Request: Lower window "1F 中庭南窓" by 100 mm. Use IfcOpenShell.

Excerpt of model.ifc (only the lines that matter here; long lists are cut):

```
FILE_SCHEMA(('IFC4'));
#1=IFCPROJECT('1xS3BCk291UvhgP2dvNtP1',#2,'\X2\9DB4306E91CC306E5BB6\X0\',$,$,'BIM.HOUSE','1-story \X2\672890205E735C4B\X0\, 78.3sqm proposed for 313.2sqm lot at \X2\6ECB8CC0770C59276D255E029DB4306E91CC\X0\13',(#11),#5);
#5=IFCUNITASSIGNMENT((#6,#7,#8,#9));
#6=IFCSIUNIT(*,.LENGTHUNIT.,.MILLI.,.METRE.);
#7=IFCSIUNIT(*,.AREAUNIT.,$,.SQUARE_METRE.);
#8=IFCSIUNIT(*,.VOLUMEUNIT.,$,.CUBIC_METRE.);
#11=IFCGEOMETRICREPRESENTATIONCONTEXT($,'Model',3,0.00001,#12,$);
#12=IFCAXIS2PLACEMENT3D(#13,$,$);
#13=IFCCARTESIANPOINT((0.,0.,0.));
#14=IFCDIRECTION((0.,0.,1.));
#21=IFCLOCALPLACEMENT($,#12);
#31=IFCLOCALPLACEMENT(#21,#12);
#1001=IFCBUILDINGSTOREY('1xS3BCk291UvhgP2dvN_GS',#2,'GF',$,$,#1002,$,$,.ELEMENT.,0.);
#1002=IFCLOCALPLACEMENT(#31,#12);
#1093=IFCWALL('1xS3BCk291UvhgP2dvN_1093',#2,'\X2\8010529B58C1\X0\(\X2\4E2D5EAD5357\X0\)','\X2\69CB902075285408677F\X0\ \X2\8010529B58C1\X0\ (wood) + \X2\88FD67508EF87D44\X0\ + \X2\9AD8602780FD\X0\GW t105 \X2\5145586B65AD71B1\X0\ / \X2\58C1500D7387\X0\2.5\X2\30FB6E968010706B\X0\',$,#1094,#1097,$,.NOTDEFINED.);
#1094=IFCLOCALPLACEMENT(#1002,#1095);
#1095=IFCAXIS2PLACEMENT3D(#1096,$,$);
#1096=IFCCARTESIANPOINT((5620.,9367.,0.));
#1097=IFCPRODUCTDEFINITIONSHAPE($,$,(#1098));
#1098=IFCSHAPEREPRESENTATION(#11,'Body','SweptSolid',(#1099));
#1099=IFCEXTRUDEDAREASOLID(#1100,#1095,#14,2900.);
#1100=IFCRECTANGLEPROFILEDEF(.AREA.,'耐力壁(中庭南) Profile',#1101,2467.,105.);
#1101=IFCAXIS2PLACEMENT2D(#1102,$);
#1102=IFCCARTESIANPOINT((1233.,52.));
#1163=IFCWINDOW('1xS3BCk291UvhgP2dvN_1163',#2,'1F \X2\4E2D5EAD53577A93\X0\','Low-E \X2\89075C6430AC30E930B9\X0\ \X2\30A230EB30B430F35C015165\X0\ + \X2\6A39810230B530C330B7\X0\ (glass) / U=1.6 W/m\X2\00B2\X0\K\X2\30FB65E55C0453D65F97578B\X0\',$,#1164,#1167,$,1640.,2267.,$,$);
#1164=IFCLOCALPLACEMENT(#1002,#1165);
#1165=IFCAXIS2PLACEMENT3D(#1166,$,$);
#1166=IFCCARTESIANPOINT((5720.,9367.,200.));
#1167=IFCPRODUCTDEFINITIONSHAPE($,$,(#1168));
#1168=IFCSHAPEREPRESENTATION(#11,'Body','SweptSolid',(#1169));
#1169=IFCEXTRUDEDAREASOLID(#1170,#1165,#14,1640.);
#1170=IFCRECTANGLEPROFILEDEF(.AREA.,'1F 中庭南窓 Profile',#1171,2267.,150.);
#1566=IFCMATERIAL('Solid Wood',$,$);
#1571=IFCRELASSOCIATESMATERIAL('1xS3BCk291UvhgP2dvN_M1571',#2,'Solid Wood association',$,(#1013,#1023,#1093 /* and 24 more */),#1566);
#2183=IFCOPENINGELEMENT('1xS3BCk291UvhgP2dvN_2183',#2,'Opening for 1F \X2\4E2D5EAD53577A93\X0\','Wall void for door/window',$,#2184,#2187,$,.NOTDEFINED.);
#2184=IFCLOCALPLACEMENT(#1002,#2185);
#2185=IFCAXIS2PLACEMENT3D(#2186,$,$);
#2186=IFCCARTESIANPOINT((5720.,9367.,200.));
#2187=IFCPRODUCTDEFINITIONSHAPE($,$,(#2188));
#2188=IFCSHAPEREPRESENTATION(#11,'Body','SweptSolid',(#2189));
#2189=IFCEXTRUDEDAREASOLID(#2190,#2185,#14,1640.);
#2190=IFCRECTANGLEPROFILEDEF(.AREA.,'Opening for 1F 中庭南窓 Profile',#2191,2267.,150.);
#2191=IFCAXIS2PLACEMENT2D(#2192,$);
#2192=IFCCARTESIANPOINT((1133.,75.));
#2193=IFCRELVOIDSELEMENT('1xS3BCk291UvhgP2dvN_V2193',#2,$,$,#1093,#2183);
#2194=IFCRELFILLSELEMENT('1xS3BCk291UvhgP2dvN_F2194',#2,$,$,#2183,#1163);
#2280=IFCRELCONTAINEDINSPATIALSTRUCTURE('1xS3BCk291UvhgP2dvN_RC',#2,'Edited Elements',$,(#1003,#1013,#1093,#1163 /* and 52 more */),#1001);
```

```python
import numpy as np
import ifcopenshell
import ifcopenshell.api.geometry
import ifcopenshell.util.placement
import ifcopenshell.util.unit

model = ifcopenshell.open("model.ifc")
unit_scale = ifcopenshell.util.unit.calculate_unit_scale(model)

window = model.by_id(1163)
opening = window.FillsVoids[0].RelatingOpeningElement
dz = -0.1 / unit_scale

shift = np.array([0.0, 0.0, dz])
# The window is not placed relative to its opening, so move both.
for product in (opening, window):
    matrix = ifcopenshell.util.placement.get_local_placement(product.ObjectPlacement)
    matrix[:3, 3] += shift
    ifcopenshell.api.geometry.edit_object_placement(model, product=product, matrix=matrix, is_si=False)

print(f"moved by {dz * unit_scale:+.3f} m")

model.write("model_rev.ifc")
```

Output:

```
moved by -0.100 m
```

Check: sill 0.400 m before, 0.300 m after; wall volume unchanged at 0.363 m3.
